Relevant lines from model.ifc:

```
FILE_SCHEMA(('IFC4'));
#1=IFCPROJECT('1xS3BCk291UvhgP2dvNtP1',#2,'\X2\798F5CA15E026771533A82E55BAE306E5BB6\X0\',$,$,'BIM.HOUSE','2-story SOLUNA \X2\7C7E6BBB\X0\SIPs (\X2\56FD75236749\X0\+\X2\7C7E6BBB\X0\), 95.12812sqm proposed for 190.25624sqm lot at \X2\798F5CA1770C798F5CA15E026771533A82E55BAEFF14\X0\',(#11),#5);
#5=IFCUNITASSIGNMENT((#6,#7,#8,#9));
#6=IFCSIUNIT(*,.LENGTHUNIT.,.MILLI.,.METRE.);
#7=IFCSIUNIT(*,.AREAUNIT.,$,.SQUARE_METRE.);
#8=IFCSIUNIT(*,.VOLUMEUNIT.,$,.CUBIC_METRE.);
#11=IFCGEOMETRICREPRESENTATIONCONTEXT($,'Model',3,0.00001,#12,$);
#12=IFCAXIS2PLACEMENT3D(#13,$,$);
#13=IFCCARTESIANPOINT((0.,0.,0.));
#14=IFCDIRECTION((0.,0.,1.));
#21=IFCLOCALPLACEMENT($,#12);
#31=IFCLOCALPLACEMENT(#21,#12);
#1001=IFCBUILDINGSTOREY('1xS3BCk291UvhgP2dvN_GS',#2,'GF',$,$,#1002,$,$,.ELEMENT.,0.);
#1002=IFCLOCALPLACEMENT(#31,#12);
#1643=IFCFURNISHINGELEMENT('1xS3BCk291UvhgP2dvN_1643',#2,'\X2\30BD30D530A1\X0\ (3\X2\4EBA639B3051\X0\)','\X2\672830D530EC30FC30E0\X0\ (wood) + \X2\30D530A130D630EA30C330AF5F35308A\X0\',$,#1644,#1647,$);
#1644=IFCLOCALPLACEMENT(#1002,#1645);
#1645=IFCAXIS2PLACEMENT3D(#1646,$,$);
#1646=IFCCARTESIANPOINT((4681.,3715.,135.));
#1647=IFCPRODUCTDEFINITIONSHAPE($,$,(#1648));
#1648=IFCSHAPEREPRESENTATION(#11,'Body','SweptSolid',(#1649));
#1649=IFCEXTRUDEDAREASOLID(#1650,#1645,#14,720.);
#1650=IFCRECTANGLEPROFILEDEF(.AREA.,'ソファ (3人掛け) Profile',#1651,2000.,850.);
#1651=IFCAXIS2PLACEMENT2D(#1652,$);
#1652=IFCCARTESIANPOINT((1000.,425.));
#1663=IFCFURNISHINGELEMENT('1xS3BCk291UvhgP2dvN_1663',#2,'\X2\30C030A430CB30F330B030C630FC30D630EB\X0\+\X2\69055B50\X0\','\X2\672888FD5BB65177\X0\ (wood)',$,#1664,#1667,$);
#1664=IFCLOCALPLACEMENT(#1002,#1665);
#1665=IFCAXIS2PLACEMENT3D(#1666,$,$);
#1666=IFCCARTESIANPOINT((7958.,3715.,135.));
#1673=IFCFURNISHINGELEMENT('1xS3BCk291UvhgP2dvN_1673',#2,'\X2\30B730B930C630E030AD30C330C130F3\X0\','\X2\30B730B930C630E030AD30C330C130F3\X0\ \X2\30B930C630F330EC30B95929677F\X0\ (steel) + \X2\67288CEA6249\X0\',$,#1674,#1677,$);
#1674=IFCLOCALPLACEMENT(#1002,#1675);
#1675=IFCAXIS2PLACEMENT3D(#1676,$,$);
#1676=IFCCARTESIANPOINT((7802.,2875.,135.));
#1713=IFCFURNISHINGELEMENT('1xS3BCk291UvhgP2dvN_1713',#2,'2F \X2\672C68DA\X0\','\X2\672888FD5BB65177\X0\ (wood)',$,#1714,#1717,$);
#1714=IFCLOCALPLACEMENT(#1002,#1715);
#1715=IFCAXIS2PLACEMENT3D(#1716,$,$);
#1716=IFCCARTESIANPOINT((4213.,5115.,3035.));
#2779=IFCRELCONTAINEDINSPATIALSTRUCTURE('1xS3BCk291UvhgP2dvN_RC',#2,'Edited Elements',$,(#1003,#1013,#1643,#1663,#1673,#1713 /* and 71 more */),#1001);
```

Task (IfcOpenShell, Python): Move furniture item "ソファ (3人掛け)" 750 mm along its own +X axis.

```python
import ifcopenshell
import ifcopenshell.api.geometry
import ifcopenshell.util.placement
import ifcopenshell.util.unit

model = ifcopenshell.open("model.ifc")
unit_scale = ifcopenshell.util.unit.calculate_unit_scale(model)

item = model.by_guid("1xS3BCk291UvhgP2dvN_1643")
matrix = ifcopenshell.util.placement.get_local_placement(item.ObjectPlacement)
matrix[:3, 3] += matrix[:3, 0] * 0.75 / unit_scale
ifcopenshell.api.geometry.edit_object_placement(model, product=item, matrix=matrix, is_si=False)

print(ifcopenshell.util.placement.get_local_placement(item.ObjectPlacement).round(3) + 0.0)

model.write("model_rev.ifc")
```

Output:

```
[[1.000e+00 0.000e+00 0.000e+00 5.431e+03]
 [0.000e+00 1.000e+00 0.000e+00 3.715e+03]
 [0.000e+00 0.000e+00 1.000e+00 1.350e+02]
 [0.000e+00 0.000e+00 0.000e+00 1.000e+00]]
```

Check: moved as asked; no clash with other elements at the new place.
